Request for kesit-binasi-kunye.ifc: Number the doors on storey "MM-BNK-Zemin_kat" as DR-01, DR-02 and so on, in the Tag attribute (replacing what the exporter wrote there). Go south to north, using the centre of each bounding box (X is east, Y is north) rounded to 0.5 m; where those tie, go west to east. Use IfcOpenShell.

First a look at what the model holds.

```python
import ifcopenshell
import ifcopenshell.util.element
import ifcopenshell.util.placement

model = ifcopenshell.open("kesit-binasi-kunye.ifc")
print(model.schema)
storey = next(s for s in model.by_type("IfcBuildingStorey") if s.Name == "MM-BNK-Zemin_kat")
doors = [e for e in ifcopenshell.util.element.get_decomposition(storey) if e.is_a("IfcDoor")]
for e in sorted(doors, key=lambda e: e.id()):
    origin = ifcopenshell.util.placement.get_local_placement(e.ObjectPlacement)[:3, 3]
    print(e.id(), e.Tag, e.Name, origin.round(2) + 0.0, sep=" | ")
```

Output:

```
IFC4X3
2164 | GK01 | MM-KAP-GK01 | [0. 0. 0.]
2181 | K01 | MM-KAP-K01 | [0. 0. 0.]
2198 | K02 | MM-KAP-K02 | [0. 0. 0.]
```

```python
import ifcopenshell
import ifcopenshell.geom
import ifcopenshell.util.element
import ifcopenshell.util.shape

model = ifcopenshell.open("kesit-binasi-kunye.ifc")
settings = ifcopenshell.geom.settings()
settings.set("use-world-coords", True)


def centre(element):
    shape = ifcopenshell.geom.create_shape(settings, element)
    return ifcopenshell.util.shape.get_bbox_centroid(shape.geometry)


storey = next(s for s in model.by_type("IfcBuildingStorey") if s.Name == "MM-BNK-Zemin_kat")
doors = [e for e in ifcopenshell.util.element.get_decomposition(storey) if e.is_a("IfcDoor")]

# Insertion points can sit at a corner or the storey origin, so sort by the geometry (in metres).
centres = {e: centre(e) for e in doors}
doors.sort(key=lambda e: (round(centres[e][1] / 0.5), centres[e][0]))

for i, e in enumerate(doors, start=1):
    number = f"DR-{i:02d}"
    e.Tag = number
    print(e.id(), number)

model.write("kesit-binasi-kunye-out.ifc")
```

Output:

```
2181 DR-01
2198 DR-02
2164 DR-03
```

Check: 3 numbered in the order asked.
